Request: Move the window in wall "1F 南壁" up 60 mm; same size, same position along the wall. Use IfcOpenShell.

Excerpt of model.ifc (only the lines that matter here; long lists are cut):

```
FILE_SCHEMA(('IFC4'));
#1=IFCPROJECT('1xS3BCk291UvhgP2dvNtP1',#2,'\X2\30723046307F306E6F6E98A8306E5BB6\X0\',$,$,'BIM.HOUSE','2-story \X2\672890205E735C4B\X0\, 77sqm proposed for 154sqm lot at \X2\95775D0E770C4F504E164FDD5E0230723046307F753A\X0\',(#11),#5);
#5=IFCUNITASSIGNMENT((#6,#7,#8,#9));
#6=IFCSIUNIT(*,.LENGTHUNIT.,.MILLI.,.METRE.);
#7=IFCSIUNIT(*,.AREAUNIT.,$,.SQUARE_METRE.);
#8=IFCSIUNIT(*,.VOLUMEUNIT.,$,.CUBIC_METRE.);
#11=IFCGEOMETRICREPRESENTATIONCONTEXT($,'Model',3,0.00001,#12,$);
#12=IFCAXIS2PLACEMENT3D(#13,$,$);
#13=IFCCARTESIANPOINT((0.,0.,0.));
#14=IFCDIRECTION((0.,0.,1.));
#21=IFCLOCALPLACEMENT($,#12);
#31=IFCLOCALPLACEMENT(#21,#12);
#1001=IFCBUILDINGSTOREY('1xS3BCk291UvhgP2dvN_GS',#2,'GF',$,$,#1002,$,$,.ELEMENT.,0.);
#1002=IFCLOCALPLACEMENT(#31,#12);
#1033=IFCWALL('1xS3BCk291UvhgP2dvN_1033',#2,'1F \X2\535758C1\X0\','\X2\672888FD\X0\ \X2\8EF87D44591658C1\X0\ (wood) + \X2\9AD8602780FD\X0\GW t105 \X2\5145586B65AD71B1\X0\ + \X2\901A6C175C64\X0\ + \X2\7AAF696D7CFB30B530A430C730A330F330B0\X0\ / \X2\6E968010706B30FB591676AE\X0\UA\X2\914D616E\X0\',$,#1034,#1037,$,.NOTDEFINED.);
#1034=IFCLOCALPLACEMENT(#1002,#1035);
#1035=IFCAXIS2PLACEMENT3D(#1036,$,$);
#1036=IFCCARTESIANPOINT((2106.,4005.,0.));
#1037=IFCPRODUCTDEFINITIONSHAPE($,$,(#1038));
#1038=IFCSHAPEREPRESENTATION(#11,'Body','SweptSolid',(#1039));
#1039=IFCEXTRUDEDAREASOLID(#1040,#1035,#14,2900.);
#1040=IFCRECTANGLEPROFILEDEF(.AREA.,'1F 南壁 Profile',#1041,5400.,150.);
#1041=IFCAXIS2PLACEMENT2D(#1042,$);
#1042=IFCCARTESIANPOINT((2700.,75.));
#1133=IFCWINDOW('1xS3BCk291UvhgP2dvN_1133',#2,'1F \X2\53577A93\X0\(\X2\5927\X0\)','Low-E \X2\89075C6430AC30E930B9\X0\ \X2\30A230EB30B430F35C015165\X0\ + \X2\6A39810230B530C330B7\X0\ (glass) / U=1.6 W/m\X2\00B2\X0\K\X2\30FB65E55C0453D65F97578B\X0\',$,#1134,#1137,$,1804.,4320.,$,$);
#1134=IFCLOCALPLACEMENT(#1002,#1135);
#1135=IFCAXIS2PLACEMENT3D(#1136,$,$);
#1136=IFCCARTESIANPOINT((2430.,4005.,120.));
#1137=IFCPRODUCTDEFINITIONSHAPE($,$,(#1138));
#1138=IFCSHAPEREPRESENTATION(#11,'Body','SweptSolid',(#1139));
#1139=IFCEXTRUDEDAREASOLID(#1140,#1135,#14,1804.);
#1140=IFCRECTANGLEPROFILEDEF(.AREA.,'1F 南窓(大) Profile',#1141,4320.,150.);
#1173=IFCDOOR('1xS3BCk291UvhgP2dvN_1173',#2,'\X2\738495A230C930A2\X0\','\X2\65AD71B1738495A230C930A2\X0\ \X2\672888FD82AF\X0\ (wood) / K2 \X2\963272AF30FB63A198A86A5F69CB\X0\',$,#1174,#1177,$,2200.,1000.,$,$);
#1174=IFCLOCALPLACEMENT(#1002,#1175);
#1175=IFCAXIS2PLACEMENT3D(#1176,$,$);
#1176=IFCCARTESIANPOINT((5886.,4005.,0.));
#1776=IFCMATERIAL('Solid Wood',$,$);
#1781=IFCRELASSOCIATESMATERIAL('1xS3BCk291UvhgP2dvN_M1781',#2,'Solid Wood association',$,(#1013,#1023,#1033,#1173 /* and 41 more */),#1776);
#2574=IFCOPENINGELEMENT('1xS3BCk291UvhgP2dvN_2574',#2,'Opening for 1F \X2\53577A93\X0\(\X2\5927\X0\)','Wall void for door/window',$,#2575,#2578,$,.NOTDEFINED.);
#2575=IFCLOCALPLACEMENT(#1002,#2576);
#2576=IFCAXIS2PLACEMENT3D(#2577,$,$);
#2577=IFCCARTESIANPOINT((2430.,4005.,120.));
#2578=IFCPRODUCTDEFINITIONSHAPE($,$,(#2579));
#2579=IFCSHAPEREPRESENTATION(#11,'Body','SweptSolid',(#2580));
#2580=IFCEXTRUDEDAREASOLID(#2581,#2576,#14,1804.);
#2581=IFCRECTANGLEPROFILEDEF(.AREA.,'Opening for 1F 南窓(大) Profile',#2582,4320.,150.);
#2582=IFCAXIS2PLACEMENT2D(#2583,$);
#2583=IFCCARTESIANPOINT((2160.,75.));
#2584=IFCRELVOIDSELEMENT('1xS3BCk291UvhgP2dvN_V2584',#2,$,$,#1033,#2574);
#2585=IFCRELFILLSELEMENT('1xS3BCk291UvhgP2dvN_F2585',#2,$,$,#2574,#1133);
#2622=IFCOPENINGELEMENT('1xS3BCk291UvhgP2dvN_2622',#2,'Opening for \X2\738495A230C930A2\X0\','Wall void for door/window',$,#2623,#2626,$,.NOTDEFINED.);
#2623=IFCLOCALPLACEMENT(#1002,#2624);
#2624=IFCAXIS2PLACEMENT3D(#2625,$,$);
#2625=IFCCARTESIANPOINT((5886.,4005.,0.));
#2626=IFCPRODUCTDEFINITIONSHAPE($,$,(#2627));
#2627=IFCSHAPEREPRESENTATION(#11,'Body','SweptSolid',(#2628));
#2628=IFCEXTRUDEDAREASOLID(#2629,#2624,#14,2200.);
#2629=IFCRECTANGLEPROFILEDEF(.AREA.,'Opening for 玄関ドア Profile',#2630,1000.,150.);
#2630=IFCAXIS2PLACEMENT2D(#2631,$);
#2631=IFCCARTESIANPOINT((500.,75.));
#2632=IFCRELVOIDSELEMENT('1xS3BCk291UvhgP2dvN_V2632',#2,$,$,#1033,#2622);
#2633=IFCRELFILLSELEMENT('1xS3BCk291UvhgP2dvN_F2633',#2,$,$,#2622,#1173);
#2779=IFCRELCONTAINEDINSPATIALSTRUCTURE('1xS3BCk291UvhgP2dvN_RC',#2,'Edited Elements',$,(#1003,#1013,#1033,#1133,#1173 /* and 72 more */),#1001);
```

```python
import numpy as np
import ifcopenshell
import ifcopenshell.api.geometry
import ifcopenshell.util.placement
import ifcopenshell.util.unit

model = ifcopenshell.open("model.ifc")
unit_scale = ifcopenshell.util.unit.calculate_unit_scale(model)

window = model.by_guid("1xS3BCk291UvhgP2dvN_1133")
opening = window.FillsVoids[0].RelatingOpeningElement
dz = 60.0

shift = np.array([0.0, 0.0, dz])
# The window is not placed relative to its opening, so move both.
for product in (opening, window):
    matrix = ifcopenshell.util.placement.get_local_placement(product.ObjectPlacement)
    matrix[:3, 3] += shift
    ifcopenshell.api.geometry.edit_object_placement(model, product=product, matrix=matrix, is_si=False)

print(f"moved by {dz * unit_scale:+.3f} m")

model.write("model_edited.ifc")
```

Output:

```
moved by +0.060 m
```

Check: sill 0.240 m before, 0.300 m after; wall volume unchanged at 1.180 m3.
